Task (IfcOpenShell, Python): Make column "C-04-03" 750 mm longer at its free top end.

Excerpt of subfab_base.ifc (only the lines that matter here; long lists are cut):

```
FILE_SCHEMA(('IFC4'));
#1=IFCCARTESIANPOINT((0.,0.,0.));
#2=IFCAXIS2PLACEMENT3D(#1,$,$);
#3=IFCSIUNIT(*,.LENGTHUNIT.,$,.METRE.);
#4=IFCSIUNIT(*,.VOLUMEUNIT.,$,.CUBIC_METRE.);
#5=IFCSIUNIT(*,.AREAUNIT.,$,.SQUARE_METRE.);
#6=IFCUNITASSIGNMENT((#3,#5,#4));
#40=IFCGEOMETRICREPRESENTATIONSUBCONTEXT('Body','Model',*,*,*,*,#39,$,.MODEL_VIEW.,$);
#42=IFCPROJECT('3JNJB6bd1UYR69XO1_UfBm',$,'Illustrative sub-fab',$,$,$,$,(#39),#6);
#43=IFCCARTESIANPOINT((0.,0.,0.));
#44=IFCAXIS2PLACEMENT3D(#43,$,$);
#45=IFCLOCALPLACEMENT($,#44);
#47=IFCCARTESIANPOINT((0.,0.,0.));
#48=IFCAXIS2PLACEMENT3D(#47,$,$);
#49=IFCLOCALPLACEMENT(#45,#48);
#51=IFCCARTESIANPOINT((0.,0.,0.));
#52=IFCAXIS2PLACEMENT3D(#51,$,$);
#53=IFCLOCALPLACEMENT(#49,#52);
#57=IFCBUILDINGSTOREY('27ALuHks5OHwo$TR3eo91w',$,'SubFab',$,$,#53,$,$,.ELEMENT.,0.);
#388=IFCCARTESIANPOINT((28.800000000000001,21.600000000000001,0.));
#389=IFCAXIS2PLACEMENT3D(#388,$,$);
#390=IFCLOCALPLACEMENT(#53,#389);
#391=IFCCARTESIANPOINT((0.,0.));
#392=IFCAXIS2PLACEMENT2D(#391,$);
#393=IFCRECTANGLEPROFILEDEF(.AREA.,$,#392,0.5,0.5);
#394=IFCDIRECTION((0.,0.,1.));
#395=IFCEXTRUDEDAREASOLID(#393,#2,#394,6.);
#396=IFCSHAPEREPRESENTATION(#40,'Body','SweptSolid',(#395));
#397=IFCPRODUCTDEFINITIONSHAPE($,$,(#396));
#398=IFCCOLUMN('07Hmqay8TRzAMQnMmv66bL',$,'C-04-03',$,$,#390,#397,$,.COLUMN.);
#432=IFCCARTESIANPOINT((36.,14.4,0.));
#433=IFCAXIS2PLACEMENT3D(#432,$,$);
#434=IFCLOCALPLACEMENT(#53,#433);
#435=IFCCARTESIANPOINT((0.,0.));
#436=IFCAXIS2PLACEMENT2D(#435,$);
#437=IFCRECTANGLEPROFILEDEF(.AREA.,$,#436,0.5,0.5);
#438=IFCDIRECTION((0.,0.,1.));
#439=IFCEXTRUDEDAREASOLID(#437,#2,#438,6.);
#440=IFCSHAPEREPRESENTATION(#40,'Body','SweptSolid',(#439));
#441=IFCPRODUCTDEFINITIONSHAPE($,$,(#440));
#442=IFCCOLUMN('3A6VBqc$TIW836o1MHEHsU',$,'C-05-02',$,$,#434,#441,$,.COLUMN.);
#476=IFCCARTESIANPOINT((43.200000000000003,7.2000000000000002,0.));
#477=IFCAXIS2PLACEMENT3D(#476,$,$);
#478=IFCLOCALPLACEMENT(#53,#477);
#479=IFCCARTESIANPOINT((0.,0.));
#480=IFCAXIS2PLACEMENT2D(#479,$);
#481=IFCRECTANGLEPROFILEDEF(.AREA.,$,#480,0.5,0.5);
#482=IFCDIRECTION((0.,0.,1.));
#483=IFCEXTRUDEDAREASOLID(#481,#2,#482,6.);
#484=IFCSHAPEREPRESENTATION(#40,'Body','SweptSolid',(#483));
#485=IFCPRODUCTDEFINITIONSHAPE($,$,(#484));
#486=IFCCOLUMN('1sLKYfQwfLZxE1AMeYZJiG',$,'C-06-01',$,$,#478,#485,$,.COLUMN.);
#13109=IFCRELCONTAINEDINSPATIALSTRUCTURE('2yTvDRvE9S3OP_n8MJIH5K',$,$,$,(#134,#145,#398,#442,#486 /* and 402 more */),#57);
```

```python
import ifcopenshell
import ifcopenshell.util.representation
import ifcopenshell.util.unit

model = ifcopenshell.open("subfab_base.ifc")
unit_scale = ifcopenshell.util.unit.calculate_unit_scale(model)

member = model.by_guid("07Hmqay8TRzAMQnMmv66bL")
change = 0.75 / unit_scale

# The extrusion runs towards the end named, so only its depth changes.
body = ifcopenshell.util.representation.get_representation(member, "Model", "Body")
solid = body.Items[0]
old_length = solid.Depth
solid.Depth += change

print(f"length {old_length:g} -> {solid.Depth:g}")

model.write("subfab_base-out.ifc")
```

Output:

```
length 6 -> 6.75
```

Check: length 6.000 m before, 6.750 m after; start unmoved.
